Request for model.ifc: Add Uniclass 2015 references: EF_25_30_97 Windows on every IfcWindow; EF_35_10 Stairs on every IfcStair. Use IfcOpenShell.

First a look at what the model holds.

```python
import ifcopenshell

model = ifcopenshell.open("model.ifc")
print(model.schema)
print("classifications:", [c.Name for c in model.by_type("IfcClassification")])
for ifc_class in ("IfcDoor", "IfcRoof", "IfcStair", "IfcWall", "IfcWindow"):
    print(ifc_class, len(model.by_type(ifc_class)))
```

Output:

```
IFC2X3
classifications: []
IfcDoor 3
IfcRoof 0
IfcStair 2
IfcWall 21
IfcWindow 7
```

```python
import ifcopenshell
import ifcopenshell.api.classification

model = ifcopenshell.open("model.ifc")

# IFC2X3 requires Source and Edition and has no link from the project to the system.
system = model.create_entity("IfcClassification", Source="NBS", Edition="2015", Name="Uniclass 2015")

codes = {
    "IfcWindow": ("EF_25_30_97", "Windows"),
    "IfcStair": ("EF_35_10", "Stairs"),
}
for ifc_class, (code, name) in codes.items():
    products = model.by_type(ifc_class)
    ifcopenshell.api.classification.add_reference(
        model, products=products, classification=system, identification=code, name=name
    )
    print(code, len(products))

model.write("model_v2.ifc")
```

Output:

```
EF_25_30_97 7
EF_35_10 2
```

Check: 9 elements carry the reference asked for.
